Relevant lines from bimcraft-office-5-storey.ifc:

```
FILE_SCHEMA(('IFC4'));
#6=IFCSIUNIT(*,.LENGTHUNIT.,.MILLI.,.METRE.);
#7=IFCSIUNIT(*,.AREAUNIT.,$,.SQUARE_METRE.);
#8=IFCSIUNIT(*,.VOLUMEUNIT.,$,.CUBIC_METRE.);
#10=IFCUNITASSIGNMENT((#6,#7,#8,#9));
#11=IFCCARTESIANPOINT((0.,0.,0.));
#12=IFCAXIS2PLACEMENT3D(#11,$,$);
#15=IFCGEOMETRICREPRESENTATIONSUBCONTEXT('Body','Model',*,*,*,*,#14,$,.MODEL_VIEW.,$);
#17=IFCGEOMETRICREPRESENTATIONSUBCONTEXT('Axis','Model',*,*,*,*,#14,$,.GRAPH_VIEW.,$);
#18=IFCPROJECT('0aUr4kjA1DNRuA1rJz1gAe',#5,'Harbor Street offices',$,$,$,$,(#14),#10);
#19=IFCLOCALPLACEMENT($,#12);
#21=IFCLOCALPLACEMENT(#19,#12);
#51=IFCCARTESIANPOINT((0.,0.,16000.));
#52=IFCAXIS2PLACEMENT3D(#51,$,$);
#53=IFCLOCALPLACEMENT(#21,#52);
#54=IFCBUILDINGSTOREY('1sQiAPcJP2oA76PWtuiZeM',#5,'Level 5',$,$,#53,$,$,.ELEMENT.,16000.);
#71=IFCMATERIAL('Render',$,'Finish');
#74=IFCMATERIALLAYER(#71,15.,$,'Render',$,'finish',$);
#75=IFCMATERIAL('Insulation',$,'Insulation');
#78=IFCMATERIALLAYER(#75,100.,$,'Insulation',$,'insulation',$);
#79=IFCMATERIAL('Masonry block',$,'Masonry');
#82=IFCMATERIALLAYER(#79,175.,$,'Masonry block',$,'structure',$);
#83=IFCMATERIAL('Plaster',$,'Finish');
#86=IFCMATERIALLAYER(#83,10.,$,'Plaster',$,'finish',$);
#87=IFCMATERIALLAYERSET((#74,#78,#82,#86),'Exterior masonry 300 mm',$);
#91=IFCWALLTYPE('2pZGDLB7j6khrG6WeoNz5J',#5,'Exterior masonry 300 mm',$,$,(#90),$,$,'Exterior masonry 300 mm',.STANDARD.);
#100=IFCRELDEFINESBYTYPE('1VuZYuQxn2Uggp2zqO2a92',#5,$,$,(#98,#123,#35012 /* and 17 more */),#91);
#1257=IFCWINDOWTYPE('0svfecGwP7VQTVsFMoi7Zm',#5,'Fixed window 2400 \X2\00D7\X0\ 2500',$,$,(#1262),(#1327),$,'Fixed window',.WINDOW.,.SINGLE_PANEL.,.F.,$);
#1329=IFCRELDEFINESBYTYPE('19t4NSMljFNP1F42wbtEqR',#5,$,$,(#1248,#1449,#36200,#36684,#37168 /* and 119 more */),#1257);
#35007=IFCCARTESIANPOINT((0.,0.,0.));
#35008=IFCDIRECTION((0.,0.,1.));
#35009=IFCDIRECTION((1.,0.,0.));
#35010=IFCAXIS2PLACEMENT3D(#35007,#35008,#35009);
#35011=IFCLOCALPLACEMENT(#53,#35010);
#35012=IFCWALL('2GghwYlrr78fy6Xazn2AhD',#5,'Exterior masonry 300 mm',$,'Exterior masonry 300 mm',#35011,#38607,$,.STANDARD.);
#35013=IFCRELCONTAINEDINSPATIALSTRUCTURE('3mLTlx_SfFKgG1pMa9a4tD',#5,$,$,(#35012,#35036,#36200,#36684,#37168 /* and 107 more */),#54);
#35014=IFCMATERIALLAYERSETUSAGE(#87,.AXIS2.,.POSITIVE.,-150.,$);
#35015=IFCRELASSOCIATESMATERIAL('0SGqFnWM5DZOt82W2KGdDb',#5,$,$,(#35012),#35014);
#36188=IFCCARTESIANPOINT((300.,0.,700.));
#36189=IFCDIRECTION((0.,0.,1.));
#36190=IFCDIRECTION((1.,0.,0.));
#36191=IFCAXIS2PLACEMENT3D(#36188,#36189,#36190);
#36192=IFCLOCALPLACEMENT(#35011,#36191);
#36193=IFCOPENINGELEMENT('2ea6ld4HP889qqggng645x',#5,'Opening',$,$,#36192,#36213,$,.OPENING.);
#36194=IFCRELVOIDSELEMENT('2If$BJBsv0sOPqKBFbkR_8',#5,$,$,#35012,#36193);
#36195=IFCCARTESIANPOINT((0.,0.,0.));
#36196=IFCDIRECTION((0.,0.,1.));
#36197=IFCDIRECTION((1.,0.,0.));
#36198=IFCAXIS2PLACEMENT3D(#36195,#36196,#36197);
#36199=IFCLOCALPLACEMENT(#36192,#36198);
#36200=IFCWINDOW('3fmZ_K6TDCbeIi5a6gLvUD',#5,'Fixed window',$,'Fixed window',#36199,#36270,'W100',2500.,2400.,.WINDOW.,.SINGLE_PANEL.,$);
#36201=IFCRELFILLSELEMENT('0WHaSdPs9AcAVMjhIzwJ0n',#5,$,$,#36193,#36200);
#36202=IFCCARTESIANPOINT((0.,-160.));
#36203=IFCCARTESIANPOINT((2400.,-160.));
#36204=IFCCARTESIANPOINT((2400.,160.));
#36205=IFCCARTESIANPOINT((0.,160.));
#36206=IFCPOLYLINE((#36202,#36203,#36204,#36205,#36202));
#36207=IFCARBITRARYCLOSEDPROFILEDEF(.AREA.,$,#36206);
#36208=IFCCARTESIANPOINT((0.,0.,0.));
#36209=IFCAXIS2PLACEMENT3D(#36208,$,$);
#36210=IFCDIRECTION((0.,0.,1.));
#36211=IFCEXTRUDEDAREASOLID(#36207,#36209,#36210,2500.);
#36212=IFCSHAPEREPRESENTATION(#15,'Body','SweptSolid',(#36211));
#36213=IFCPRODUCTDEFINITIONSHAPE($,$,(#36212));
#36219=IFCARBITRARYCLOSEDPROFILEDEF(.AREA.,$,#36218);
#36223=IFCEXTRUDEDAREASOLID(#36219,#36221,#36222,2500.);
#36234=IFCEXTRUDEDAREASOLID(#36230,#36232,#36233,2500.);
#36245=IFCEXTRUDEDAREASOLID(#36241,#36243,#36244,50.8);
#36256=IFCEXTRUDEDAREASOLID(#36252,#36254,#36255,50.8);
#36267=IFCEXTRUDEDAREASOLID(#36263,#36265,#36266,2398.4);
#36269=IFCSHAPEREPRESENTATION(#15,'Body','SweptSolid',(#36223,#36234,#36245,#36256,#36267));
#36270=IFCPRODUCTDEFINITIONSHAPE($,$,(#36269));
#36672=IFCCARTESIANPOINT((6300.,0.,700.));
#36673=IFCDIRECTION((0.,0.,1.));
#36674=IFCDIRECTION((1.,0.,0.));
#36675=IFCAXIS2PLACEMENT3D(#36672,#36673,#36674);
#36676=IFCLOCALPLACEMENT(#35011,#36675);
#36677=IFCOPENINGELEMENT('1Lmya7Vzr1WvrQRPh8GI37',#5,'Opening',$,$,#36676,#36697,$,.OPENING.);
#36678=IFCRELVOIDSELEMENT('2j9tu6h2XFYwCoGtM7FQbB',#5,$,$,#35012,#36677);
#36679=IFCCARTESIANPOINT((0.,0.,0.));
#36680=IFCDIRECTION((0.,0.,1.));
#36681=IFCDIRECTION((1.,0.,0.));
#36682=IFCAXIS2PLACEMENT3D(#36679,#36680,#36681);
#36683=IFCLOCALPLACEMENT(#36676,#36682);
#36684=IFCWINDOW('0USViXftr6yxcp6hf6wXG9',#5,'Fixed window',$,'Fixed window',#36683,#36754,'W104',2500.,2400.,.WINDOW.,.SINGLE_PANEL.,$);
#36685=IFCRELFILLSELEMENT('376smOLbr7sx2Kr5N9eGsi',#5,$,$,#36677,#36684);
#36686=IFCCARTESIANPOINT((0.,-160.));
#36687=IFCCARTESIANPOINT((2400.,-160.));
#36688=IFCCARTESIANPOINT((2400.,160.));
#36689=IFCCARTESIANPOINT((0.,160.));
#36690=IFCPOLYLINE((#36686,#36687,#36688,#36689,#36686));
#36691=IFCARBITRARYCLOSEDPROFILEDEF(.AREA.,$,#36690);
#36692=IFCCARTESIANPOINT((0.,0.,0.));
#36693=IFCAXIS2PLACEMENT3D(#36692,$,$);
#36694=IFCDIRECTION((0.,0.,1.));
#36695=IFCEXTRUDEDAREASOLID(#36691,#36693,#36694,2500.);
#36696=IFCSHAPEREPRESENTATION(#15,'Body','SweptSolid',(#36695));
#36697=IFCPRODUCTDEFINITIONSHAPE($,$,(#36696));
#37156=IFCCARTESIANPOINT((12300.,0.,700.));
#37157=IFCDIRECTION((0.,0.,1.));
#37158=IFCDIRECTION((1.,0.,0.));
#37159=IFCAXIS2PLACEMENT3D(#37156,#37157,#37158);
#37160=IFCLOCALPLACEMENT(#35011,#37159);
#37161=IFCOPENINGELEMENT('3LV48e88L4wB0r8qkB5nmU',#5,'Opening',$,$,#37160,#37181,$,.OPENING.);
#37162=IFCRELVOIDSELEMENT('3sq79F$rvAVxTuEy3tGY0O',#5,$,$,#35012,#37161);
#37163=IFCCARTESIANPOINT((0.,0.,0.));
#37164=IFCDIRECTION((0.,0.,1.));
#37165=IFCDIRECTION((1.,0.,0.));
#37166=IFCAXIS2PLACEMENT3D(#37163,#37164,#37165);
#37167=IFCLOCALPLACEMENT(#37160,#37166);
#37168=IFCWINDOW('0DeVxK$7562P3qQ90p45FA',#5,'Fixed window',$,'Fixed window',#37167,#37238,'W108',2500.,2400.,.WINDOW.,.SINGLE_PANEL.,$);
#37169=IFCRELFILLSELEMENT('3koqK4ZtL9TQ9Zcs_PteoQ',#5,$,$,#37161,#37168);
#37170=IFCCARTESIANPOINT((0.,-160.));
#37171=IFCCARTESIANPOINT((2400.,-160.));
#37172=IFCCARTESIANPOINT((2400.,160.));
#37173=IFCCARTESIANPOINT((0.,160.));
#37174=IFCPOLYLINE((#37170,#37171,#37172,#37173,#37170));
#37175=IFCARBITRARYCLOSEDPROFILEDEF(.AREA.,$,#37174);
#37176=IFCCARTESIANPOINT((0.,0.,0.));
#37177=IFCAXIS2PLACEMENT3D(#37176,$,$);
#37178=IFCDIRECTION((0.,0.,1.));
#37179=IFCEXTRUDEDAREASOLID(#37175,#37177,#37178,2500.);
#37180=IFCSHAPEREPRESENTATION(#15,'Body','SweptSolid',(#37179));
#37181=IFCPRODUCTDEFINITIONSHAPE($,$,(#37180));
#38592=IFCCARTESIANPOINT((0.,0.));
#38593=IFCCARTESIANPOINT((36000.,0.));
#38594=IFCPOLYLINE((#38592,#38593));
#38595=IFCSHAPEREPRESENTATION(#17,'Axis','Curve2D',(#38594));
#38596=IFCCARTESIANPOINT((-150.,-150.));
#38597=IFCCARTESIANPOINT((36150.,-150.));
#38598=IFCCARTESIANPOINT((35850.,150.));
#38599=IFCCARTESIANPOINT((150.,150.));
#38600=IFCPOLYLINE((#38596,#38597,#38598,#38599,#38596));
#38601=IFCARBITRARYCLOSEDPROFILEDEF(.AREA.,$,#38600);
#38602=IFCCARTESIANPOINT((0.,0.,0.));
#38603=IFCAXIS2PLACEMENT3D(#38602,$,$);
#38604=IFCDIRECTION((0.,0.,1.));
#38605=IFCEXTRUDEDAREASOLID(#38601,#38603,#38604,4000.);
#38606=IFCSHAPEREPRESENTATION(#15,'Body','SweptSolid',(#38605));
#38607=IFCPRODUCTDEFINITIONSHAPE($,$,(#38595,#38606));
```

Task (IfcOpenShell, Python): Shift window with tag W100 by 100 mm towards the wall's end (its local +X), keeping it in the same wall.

```python
import ifcopenshell
import ifcopenshell.api.geometry
import ifcopenshell.util.placement
import ifcopenshell.util.unit

model = ifcopenshell.open("bimcraft-office-5-storey.ifc")
unit_scale = ifcopenshell.util.unit.calculate_unit_scale(model)

window = model.by_guid("3fmZ_K6TDCbeIi5a6gLvUD")
opening = window.FillsVoids[0].RelatingOpeningElement
wall = opening.VoidsElements[0].RelatingBuildingElement

wall_matrix = ifcopenshell.util.placement.get_local_placement(wall.ObjectPlacement)
shift = wall_matrix[:3, 0] * 0.1 / unit_scale
before = ifcopenshell.util.placement.get_local_placement(window.ObjectPlacement)[:3, 3].copy()

# The window is placed relative to its opening, so it follows when the opening moves.
matrix = ifcopenshell.util.placement.get_local_placement(opening.ObjectPlacement)
matrix[:3, 3] += shift
ifcopenshell.api.geometry.edit_object_placement(
    model, product=opening, matrix=matrix, is_si=False, should_transform_children=True
)

after = ifcopenshell.util.placement.get_local_placement(window.ObjectPlacement)[:3, 3]
print("window moved by", (after - before).round(3) + 0.0)

model.write("bimcraft-office-5-storey-out.ifc")
```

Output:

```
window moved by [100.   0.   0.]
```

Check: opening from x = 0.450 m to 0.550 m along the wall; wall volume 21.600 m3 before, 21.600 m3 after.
